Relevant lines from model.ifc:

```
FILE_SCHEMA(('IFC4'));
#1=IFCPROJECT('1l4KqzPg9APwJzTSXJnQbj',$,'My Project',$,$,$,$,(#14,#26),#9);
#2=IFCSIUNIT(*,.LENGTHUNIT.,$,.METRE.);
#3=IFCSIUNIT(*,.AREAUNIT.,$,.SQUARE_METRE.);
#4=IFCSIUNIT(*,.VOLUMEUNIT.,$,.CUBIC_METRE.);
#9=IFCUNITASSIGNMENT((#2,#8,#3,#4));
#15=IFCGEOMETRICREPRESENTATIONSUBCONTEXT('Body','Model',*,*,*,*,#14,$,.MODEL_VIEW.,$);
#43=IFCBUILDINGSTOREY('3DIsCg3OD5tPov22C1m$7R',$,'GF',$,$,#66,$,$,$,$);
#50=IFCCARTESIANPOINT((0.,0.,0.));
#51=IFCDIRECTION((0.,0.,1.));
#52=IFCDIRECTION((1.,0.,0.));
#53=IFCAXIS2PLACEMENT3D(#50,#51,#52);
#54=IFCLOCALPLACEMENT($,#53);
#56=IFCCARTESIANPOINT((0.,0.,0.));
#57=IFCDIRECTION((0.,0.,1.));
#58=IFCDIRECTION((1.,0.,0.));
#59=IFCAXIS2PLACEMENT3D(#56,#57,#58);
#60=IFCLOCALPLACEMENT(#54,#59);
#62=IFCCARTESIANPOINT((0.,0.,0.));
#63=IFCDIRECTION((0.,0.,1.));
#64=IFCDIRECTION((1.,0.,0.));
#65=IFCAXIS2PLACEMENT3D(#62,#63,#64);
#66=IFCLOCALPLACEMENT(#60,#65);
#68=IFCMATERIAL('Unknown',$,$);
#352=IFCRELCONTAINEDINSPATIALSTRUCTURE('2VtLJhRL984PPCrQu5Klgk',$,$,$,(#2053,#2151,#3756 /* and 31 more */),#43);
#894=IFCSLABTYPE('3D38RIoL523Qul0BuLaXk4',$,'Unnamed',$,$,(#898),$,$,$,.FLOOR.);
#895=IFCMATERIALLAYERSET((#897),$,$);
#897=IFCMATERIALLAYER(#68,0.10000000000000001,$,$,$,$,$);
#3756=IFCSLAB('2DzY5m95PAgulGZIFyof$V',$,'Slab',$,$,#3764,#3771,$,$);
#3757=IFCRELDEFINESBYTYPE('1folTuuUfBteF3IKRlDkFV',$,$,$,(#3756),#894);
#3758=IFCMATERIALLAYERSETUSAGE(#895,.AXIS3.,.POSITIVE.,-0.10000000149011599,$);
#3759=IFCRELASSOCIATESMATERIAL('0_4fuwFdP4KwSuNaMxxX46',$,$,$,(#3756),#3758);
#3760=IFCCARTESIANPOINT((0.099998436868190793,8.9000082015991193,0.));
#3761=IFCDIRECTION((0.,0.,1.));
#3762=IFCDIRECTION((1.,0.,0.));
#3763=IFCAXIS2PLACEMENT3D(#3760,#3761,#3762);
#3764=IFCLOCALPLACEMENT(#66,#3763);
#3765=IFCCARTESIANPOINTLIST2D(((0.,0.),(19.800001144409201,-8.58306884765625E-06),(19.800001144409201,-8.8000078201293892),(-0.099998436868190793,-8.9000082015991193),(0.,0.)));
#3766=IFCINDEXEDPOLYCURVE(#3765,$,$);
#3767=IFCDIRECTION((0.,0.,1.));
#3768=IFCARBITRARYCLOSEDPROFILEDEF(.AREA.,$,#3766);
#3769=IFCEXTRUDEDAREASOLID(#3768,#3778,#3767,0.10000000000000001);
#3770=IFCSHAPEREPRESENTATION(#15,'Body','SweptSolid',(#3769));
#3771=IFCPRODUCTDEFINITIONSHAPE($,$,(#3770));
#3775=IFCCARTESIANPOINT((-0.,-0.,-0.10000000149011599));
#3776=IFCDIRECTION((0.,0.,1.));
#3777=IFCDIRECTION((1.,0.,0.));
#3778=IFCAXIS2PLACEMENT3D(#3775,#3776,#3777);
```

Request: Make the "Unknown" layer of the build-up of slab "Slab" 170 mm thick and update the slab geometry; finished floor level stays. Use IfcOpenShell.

```python
import ifcopenshell
import ifcopenshell.util.element
import ifcopenshell.util.representation
import ifcopenshell.util.unit

model = ifcopenshell.open("model.ifc")
unit_scale = ifcopenshell.util.unit.calculate_unit_scale(model)

layer_set = model.by_id(895)
layer = next(l for l in layer_set.MaterialLayers if l.Material and l.Material.Name == "Unknown")
change = 0.17 / unit_scale - layer.LayerThickness
layer.LayerThickness += change

# Geometry does not follow the layer set by itself.
slabs = [e for e in ifcopenshell.util.element.get_elements_by_material(model, layer_set) if e.is_a("IfcSlab")]
for slab in sorted(slabs, key=lambda e: e.id()):
    body = ifcopenshell.util.representation.get_representation(slab, "Model", "Body")
    solid = body.Items[0]
    old_depth = solid.Depth
    solid.Depth += change
    # Extruded upwards: lower the start of the extrusion so the top stays.
    x, y, z = solid.Position.Location.Coordinates
    solid.Position.Location = model.createIfcCartesianPoint((x, y, z - change))
    print(slab.id(), f"{old_depth:g} -> {solid.Depth:g}")

# The layers are counted up from the underside, which has moved.
for usage in {ifcopenshell.util.element.get_material(slab) for slab in slabs}:
    usage.OffsetFromReferenceLine -= change

model.write("model_edited.ifc")
```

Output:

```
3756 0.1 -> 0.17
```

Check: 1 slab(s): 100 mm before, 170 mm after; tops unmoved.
